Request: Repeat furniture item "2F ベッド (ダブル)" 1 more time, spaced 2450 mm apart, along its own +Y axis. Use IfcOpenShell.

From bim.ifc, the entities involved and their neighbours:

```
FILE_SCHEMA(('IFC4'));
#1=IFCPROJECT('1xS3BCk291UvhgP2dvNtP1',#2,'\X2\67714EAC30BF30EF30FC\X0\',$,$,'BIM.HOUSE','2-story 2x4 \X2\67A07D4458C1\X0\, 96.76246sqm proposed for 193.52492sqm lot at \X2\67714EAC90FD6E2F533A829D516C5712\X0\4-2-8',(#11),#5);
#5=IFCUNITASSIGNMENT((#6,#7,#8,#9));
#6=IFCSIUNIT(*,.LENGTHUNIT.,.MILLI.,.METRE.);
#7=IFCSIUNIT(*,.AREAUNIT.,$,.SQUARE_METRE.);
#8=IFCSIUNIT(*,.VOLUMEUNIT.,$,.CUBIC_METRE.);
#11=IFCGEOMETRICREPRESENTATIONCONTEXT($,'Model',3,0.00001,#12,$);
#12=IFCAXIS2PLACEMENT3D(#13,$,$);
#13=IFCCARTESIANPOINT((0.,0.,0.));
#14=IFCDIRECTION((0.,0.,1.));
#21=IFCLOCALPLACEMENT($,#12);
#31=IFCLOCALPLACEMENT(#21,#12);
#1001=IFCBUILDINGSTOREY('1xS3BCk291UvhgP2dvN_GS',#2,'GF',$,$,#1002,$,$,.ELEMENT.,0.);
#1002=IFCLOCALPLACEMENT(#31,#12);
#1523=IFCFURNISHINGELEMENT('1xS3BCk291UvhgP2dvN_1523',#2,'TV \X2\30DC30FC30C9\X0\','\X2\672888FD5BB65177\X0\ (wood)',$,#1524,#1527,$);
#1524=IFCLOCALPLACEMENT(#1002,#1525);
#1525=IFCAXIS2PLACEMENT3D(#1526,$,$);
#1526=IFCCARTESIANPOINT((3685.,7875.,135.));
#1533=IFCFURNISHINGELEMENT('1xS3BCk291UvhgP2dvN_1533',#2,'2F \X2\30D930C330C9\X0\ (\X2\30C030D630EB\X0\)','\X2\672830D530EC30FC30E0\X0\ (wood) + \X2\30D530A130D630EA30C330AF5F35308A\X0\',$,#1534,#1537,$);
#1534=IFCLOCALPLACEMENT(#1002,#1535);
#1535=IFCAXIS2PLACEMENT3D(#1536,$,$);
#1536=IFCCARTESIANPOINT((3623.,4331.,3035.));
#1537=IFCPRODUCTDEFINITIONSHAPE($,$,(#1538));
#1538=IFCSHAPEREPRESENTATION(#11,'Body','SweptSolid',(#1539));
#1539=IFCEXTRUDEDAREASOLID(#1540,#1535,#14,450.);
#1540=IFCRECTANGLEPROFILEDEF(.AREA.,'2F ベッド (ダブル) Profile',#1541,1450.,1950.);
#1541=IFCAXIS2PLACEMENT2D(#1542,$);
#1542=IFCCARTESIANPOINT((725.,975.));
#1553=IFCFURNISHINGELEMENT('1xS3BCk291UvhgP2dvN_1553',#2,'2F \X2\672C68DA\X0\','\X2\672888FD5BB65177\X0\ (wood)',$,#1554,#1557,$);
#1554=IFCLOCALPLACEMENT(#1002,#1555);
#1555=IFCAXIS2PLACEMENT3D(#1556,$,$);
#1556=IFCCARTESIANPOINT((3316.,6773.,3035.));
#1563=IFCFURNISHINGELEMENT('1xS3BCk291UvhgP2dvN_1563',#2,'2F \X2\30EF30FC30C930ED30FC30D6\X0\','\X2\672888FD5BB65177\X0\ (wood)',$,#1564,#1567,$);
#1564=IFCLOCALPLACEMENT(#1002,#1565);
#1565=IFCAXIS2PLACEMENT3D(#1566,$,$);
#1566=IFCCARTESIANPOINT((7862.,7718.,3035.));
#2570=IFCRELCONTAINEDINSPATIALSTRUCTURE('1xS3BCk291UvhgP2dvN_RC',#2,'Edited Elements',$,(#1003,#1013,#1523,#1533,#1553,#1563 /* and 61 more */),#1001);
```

```python
import ifcopenshell
import ifcopenshell.api.geometry
import ifcopenshell.api.root
import ifcopenshell.util.element
import ifcopenshell.util.placement
import ifcopenshell.util.unit

model = ifcopenshell.open("bim.ifc")
unit_scale = ifcopenshell.util.unit.calculate_unit_scale(model)


def reuse_history(source, copy):
    """copy_class also copies each property set's owner history, people and application; keep the originals."""
    for rel in copy.IsDefinedBy:
        if rel.is_a("IfcRelDefinesByProperties") and (history := rel.RelatingPropertyDefinition.OwnerHistory):
            rel.RelatingPropertyDefinition.OwnerHistory = source.OwnerHistory
            ifcopenshell.util.element.remove_deep2(model, history)


source = model.by_guid("1xS3BCk291UvhgP2dvN_1533")
base = ifcopenshell.util.placement.get_local_placement(source.ObjectPlacement)
step = base[:3, 1] * 2.45 / unit_scale

for i in range(1, 2):
    copy = ifcopenshell.api.root.copy_class(model, product=source)
    copy.Representation = ifcopenshell.util.element.copy_deep(
        model, source.Representation, exclude=["IfcGeometricRepresentationContext", "IfcRepresentationMap"]
    )
    reuse_history(source, copy)
    matrix = base.copy()
    matrix[:3, 3] += i * step
    print("added at", matrix[:3, 3].round(3) + 0.0)
    ifcopenshell.api.geometry.edit_object_placement(model, product=copy, matrix=matrix, is_si=False)

model.write("bim_v2.ifc")
```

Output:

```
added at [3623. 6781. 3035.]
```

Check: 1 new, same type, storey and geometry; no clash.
